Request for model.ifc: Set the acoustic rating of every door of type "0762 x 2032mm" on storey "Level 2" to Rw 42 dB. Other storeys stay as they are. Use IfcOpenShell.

First a look at what the model holds.

```python
import ifcopenshell
import ifcopenshell.util.element

model = ifcopenshell.open("model.ifc")
print(model.schema)
storey = next(s for s in model.by_type("IfcBuildingStorey") if s.Name == "Level 2")
doors = [e for e in ifcopenshell.util.element.get_decomposition(storey) if e.is_a("IfcDoor")]
seen = {}
for e in doors:
    element_type = ifcopenshell.util.element.get_type(e)
    key = (element_type.Name if element_type != e and element_type else None, ifcopenshell.util.element.get_pset(e, "Pset_DoorCommon", "AcousticRating"))
    seen[key] = seen.get(key, 0) + 1
for (name, value), count in sorted(seen.items(), key=str):
    print(count, "x", name, "|", value)
```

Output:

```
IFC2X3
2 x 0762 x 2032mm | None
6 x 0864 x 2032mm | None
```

```python
import ifcopenshell
import ifcopenshell.api.pset
import ifcopenshell.util.element

model = ifcopenshell.open("model.ifc")

storey = next(s for s in model.by_type("IfcBuildingStorey") if s.Name == "Level 2")
doors = [e for e in ifcopenshell.util.element.get_decomposition(storey) if e.is_a("IfcDoor")]

count = 0
for e in doors:
    element_type = ifcopenshell.util.element.get_type(e)
    if element_type in (None, e) or element_type.Name != "0762 x 2032mm":
        continue
    # add_pset returns the element's existing set when there is one.
    pset = ifcopenshell.api.pset.add_pset(model, product=e, name="Pset_DoorCommon")
    ifcopenshell.api.pset.edit_pset(model, pset=pset, properties={"AcousticRating": "Rw 42 dB"})
    count += 1

print(count, "doors updated")

model.write("model_edited.ifc")
```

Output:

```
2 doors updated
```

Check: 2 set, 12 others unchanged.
